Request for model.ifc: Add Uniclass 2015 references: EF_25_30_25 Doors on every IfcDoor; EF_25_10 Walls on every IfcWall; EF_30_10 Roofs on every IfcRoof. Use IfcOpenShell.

First a look at what the model holds.

```python
import ifcopenshell

model = ifcopenshell.open("model.ifc")
print(model.schema)
print("classifications:", [c.Name for c in model.by_type("IfcClassification")])
for ifc_class in ("IfcDoor", "IfcRoof", "IfcStair", "IfcWall", "IfcWindow"):
    print(ifc_class, len(model.by_type(ifc_class)))
```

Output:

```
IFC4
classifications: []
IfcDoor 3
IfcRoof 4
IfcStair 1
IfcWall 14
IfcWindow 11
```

```python
import ifcopenshell
import ifcopenshell.api.classification

model = ifcopenshell.open("model.ifc")

system = ifcopenshell.api.classification.add_classification(model, classification="Uniclass 2015")

codes = {
    "IfcDoor": ("EF_25_30_25", "Doors"),
    "IfcWall": ("EF_25_10", "Walls"),
    "IfcRoof": ("EF_30_10", "Roofs"),
}
for ifc_class, (code, name) in codes.items():
    products = model.by_type(ifc_class)
    ifcopenshell.api.classification.add_reference(
        model, products=products, classification=system, identification=code, name=name
    )
    print(code, len(products))

model.write("model_edited.ifc")
```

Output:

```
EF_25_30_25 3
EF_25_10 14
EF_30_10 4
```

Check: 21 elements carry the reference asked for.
